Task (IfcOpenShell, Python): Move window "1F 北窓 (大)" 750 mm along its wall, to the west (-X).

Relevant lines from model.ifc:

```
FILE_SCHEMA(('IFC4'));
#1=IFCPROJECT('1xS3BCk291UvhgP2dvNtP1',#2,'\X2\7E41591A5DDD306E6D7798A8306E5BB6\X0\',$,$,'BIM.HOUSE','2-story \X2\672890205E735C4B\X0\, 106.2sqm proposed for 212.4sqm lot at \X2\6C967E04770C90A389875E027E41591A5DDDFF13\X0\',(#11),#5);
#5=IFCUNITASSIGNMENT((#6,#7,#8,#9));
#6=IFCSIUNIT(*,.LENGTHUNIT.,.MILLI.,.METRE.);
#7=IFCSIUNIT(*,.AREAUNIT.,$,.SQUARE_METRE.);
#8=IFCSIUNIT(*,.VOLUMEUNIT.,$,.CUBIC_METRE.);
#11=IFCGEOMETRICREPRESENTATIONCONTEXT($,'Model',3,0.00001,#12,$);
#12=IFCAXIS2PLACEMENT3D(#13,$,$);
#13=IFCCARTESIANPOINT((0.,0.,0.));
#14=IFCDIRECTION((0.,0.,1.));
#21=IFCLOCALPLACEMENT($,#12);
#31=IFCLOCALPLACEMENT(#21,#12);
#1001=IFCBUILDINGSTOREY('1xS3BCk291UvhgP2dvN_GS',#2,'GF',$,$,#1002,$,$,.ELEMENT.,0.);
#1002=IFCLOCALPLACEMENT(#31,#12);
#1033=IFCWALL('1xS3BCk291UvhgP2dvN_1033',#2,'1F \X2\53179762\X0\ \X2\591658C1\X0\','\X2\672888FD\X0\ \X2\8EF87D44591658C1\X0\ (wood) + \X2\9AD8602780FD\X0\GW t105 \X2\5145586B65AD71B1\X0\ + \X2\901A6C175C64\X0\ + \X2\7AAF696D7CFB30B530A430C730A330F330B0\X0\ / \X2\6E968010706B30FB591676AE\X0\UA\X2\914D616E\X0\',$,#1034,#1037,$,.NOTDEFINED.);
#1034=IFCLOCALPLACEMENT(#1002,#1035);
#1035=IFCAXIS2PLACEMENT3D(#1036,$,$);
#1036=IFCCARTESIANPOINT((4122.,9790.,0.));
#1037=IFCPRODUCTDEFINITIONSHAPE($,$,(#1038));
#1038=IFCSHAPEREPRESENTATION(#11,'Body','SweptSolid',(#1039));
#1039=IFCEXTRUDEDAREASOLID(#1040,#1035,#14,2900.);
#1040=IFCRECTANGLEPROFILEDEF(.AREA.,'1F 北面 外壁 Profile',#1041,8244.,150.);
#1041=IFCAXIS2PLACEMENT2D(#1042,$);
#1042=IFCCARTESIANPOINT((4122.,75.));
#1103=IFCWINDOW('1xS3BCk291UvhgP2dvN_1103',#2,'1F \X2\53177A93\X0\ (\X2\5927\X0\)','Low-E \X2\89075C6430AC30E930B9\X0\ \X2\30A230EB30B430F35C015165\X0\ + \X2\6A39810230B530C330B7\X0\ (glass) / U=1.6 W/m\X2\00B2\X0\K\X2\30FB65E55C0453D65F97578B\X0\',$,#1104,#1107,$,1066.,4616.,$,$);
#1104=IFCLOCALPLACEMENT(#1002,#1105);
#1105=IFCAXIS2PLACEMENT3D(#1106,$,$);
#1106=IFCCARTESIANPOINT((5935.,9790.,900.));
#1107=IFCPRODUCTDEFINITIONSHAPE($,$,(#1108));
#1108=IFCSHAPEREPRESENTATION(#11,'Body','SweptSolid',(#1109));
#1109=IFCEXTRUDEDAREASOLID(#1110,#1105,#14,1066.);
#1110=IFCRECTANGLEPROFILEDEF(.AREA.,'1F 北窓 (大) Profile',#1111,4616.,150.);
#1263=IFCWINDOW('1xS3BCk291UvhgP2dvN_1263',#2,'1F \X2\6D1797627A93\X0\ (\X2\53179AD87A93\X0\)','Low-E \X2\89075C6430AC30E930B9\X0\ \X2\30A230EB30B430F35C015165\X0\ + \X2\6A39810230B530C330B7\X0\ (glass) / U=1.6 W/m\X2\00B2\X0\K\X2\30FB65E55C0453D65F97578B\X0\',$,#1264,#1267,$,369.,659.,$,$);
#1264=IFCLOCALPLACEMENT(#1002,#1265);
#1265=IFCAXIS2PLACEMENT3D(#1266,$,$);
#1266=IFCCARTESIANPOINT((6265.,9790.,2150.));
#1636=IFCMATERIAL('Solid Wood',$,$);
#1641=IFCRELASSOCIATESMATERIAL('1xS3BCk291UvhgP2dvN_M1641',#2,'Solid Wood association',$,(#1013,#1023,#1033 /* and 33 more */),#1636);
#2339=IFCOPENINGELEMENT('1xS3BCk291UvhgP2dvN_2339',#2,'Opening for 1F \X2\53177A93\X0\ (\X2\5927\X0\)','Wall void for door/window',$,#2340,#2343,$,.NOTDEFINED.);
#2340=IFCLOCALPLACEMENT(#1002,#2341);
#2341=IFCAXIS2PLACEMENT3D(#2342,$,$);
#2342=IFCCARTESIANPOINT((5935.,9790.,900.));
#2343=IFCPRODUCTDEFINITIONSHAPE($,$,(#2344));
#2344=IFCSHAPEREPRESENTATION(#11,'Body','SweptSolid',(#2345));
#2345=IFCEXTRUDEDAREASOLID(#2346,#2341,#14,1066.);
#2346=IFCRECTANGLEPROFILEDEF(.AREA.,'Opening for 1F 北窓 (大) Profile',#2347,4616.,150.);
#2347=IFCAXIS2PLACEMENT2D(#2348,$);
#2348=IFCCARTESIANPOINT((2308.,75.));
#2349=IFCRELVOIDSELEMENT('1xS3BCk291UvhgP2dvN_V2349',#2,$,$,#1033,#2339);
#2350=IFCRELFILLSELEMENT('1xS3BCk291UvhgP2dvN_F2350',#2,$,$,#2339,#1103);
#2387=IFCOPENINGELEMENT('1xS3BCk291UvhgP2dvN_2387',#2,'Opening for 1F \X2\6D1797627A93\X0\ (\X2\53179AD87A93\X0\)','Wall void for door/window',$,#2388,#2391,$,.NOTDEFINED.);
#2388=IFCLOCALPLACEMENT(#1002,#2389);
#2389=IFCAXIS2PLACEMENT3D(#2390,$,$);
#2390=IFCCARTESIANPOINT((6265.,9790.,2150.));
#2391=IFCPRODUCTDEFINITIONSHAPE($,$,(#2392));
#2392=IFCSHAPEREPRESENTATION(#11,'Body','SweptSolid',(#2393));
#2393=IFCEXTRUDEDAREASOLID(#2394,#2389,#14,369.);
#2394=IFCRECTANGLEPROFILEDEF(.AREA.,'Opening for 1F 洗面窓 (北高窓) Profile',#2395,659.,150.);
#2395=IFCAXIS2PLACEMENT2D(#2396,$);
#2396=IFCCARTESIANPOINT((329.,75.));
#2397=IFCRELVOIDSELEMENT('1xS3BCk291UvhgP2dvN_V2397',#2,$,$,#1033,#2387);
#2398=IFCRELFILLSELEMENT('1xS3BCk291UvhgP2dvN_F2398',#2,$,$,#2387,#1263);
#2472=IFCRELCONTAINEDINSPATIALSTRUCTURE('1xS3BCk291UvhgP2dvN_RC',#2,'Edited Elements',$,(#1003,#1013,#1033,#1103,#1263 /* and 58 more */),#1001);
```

```python
import ifcopenshell
import ifcopenshell.api.geometry
import ifcopenshell.util.placement

model = ifcopenshell.open("model.ifc")

window = model.by_guid("1xS3BCk291UvhgP2dvN_1103")
opening = window.FillsVoids[0].RelatingOpeningElement
wall = opening.VoidsElements[0].RelatingBuildingElement

wall_matrix = ifcopenshell.util.placement.get_local_placement(wall.ObjectPlacement)
shift = wall_matrix[:3, 0] * -750.0
before = ifcopenshell.util.placement.get_local_placement(window.ObjectPlacement)[:3, 3].copy()

# The window is not placed relative to its opening, so move both.
for product in (opening, window):
    matrix = ifcopenshell.util.placement.get_local_placement(product.ObjectPlacement)
    matrix[:3, 3] += shift
    ifcopenshell.api.geometry.edit_object_placement(model, product=product, matrix=matrix, is_si=False)

after = ifcopenshell.util.placement.get_local_placement(window.ObjectPlacement)[:3, 3]
print("window moved by", (after - before).round(3) + 0.0)

model.write("model_v2.ifc")
```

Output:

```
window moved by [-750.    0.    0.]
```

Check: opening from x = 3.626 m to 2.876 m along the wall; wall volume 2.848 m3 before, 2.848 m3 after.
